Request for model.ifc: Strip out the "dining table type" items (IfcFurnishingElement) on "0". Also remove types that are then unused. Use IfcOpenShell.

First a look at what the model holds.

```python
import ifcopenshell
import ifcopenshell.util.element

model = ifcopenshell.open("model.ifc")
print(model.schema)
storey = next(s for s in model.by_type("IfcBuildingStorey") if s.Name == "0")
furniture = [e for e in ifcopenshell.util.element.get_decomposition(storey) if e.is_a("IfcFurnishingElement")]
seen = {}
for e in furniture:
    element_type = ifcopenshell.util.element.get_type(e)
    name = element_type.Name if element_type not in (None, e) else None
    seen[name] = seen.get(name, 0) + 1
for name, count in sorted(seen.items(), key=str):
    print(count, "x", name)
```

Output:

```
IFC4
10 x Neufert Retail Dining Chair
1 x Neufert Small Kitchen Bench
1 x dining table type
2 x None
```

```python
import ifcopenshell
import ifcopenshell.api.root
import ifcopenshell.util.element

model = ifcopenshell.open("model.ifc")

storey = next(s for s in model.by_type("IfcBuildingStorey") if s.Name == "0")
furniture = [e for e in ifcopenshell.util.element.get_decomposition(storey) if e.is_a("IfcFurnishingElement")]
targets = [e for e in furniture if (t := ifcopenshell.util.element.get_type(e)) not in (None, e) and t.Name == "dining table type"]
types = {ifcopenshell.util.element.get_type(e) for e in targets} - {None, *targets}

for e in targets:
    ifcopenshell.api.root.remove_product(model, product=e)
print(len(targets), "removed")

unused = [t for t in types if not ifcopenshell.util.element.get_types(t)]
for t in unused:
    ifcopenshell.api.root.remove_product(model, product=t)
print(len(unused), "unused types removed")

model.write("model_rev.ifc")
```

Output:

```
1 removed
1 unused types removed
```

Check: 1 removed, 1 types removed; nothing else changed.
